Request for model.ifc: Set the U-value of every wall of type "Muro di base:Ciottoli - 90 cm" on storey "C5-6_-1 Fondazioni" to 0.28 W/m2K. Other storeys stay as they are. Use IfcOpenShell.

First a look at what the model holds.

```python
import ifcopenshell
import ifcopenshell.util.element

model = ifcopenshell.open("model.ifc")
print(model.schema)
storey = next(s for s in model.by_type("IfcBuildingStorey") if s.Name == "C5-6_-1 Fondazioni")
walls = [e for e in ifcopenshell.util.element.get_decomposition(storey) if e.is_a("IfcWall")]
seen = {}
for e in walls:
    element_type = ifcopenshell.util.element.get_type(e)
    key = (element_type.Name if element_type != e and element_type else None, ifcopenshell.util.element.get_pset(e, "Pset_WallCommon", "ThermalTransmittance"))
    seen[key] = seen.get(key, 0) + 1
for (name, value), count in sorted(seen.items(), key=str):
    print(count, "x", name, "|", value)
```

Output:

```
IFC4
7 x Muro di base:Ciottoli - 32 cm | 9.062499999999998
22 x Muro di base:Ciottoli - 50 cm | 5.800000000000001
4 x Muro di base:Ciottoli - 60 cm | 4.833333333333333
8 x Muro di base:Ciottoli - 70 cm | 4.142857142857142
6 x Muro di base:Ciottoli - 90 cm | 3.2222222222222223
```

```python
import ifcopenshell
import ifcopenshell.api.pset
import ifcopenshell.util.element

model = ifcopenshell.open("model.ifc")

storey = next(s for s in model.by_type("IfcBuildingStorey") if s.Name == "C5-6_-1 Fondazioni")
walls = [e for e in ifcopenshell.util.element.get_decomposition(storey) if e.is_a("IfcWall")]

count = 0
for e in walls:
    element_type = ifcopenshell.util.element.get_type(e)
    if element_type in (None, e) or element_type.Name != "Muro di base:Ciottoli - 90 cm":
        continue
    # add_pset returns the element's existing set when there is one.
    pset = ifcopenshell.api.pset.add_pset(model, product=e, name="Pset_WallCommon")
    ifcopenshell.api.pset.edit_pset(model, pset=pset, properties={"ThermalTransmittance": 0.28})
    count += 1

print(count, "walls updated")

model.write("model_edited.ifc")
```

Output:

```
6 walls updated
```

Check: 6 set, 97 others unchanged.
